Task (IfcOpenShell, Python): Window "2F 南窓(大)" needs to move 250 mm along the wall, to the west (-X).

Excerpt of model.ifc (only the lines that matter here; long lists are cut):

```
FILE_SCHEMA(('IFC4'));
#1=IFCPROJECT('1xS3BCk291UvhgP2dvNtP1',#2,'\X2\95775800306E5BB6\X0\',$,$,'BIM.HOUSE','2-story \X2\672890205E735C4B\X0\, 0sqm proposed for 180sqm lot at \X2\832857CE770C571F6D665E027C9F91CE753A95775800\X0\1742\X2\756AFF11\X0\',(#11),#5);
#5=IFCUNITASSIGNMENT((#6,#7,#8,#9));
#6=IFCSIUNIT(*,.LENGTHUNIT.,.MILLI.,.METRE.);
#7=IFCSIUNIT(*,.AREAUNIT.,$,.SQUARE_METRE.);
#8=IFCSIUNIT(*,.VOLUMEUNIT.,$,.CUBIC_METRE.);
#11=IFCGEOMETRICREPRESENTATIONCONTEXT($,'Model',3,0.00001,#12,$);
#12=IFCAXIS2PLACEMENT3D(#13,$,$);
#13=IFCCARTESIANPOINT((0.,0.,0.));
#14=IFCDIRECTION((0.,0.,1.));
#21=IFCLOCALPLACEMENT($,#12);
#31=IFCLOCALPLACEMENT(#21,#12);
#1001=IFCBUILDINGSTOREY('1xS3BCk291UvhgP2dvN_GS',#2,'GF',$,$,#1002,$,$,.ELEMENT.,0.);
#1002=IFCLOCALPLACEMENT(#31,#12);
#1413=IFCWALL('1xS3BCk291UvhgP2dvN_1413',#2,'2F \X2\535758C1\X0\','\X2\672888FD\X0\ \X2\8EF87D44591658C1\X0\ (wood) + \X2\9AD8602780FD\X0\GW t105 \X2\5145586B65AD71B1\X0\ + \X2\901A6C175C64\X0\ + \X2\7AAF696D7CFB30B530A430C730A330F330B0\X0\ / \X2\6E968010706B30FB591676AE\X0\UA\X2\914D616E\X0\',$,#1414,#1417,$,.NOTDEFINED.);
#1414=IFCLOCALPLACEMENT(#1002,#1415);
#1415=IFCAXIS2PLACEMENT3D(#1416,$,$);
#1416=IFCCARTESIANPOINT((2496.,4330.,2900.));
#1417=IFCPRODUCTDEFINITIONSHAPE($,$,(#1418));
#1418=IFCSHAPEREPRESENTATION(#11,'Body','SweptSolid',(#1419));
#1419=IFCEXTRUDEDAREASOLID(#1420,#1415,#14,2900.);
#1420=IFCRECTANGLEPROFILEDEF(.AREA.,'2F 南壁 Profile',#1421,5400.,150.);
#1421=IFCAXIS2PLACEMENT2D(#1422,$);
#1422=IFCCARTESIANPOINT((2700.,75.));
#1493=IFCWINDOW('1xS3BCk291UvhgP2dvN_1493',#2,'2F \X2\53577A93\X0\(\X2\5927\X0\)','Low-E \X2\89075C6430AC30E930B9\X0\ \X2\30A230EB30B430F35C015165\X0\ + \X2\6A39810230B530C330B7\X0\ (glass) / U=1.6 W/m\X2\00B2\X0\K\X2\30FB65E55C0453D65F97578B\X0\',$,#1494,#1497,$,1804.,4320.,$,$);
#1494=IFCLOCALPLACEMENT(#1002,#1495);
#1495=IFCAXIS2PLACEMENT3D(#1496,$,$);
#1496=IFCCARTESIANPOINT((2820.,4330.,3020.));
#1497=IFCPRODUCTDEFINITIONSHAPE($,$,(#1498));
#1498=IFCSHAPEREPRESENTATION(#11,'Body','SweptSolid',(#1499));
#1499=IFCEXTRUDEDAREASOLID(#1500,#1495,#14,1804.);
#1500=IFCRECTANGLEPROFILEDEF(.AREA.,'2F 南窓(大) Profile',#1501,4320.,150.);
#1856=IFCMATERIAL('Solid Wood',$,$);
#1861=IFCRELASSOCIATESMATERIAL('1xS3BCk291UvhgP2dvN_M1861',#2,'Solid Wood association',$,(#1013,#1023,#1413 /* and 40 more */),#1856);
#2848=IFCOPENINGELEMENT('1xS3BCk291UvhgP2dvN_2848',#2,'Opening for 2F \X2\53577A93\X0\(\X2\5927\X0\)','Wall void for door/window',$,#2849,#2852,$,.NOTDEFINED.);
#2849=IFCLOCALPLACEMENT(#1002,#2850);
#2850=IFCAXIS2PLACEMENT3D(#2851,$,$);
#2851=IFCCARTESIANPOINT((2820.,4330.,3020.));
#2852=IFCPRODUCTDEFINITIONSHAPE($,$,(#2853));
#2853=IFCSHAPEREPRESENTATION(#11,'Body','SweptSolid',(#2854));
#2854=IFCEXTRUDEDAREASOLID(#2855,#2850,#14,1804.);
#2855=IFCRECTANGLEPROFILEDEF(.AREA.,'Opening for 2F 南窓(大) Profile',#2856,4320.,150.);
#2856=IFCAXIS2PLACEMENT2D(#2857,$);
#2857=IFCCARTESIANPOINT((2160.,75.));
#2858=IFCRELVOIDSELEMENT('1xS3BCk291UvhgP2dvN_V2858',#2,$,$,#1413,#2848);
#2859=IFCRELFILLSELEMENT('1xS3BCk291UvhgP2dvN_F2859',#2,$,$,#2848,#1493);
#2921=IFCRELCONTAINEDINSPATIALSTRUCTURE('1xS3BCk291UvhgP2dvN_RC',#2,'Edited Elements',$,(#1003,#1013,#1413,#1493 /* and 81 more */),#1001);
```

```python
import ifcopenshell
import ifcopenshell.api.geometry
import ifcopenshell.util.placement
import ifcopenshell.util.unit

model = ifcopenshell.open("model.ifc")
unit_scale = ifcopenshell.util.unit.calculate_unit_scale(model)

window = model.by_id(1493)
opening = window.FillsVoids[0].RelatingOpeningElement
wall = opening.VoidsElements[0].RelatingBuildingElement

wall_matrix = ifcopenshell.util.placement.get_local_placement(wall.ObjectPlacement)
shift = wall_matrix[:3, 0] * -0.25 / unit_scale
before = ifcopenshell.util.placement.get_local_placement(window.ObjectPlacement)[:3, 3].copy()

# The window is not placed relative to its opening, so move both.
for product in (opening, window):
    matrix = ifcopenshell.util.placement.get_local_placement(product.ObjectPlacement)
    matrix[:3, 3] += shift
    ifcopenshell.api.geometry.edit_object_placement(model, product=product, matrix=matrix, is_si=False)

after = ifcopenshell.util.placement.get_local_placement(window.ObjectPlacement)[:3, 3]
print("window moved by", (after - before).round(3) + 0.0)

model.write("model_rev.ifc")
```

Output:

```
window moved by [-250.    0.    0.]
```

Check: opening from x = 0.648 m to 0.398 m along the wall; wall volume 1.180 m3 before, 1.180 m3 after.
